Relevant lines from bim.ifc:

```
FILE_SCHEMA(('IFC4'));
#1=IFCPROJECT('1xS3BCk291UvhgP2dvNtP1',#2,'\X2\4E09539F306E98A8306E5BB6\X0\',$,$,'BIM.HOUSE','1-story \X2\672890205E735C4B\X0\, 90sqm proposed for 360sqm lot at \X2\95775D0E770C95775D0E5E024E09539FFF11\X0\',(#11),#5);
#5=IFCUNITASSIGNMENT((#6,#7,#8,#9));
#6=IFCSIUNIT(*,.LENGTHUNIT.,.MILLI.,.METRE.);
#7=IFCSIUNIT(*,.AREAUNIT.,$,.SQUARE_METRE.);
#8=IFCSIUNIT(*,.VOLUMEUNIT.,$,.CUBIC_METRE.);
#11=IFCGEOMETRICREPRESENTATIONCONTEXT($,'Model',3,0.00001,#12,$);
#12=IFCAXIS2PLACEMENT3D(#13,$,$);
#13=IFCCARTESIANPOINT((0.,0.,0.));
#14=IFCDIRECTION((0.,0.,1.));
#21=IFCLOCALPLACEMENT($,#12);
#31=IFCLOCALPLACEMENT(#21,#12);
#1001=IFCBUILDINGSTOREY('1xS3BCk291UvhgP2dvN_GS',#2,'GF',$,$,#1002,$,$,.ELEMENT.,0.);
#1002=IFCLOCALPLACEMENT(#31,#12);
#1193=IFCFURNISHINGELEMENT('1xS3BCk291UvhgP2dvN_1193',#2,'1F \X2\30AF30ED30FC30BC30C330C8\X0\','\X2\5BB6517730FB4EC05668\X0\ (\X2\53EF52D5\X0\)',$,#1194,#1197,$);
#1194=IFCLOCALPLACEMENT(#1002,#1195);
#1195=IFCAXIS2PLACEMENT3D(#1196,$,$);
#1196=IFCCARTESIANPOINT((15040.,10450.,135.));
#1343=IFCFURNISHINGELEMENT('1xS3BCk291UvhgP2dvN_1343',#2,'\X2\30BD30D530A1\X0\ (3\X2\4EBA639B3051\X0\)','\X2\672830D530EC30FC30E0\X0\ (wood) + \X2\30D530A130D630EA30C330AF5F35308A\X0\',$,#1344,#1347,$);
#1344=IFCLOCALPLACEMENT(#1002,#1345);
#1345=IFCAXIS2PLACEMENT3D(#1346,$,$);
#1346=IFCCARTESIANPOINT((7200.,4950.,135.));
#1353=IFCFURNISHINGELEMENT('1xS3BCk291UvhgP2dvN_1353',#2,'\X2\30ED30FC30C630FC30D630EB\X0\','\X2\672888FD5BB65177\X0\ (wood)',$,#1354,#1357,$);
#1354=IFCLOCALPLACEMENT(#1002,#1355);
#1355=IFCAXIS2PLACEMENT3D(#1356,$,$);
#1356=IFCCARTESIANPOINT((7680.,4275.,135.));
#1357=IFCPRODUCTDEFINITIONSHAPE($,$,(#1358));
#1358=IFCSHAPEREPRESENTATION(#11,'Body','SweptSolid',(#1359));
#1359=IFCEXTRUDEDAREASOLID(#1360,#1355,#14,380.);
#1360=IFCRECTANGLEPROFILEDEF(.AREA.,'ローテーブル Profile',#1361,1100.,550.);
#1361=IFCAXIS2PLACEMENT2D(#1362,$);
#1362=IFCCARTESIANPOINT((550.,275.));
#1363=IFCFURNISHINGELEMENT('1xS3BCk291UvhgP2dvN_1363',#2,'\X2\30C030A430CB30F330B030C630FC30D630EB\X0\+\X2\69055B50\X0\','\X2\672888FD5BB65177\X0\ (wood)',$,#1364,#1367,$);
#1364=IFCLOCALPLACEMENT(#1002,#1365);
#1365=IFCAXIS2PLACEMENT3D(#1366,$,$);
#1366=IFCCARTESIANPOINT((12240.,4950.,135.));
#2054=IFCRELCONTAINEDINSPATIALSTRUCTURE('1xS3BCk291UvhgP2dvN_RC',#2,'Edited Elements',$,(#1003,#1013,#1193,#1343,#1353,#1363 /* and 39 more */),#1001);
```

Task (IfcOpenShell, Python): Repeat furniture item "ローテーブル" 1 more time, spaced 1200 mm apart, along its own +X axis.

```python
import ifcopenshell
import ifcopenshell.api.geometry
import ifcopenshell.api.root
import ifcopenshell.util.element
import ifcopenshell.util.placement

model = ifcopenshell.open("bim.ifc")


def reuse_history(source, copy):
    """copy_class also copies each property set's owner history, people and application; keep the originals."""
    for rel in copy.IsDefinedBy:
        if rel.is_a("IfcRelDefinesByProperties") and (history := rel.RelatingPropertyDefinition.OwnerHistory):
            rel.RelatingPropertyDefinition.OwnerHistory = source.OwnerHistory
            ifcopenshell.util.element.remove_deep2(model, history)


source = model.by_id(1353)
base = ifcopenshell.util.placement.get_local_placement(source.ObjectPlacement)
step = base[:3, 0] * 1200.0

for i in range(1, 2):
    copy = ifcopenshell.api.root.copy_class(model, product=source)
    copy.Representation = ifcopenshell.util.element.copy_deep(
        model, source.Representation, exclude=["IfcGeometricRepresentationContext", "IfcRepresentationMap"]
    )
    reuse_history(source, copy)
    matrix = base.copy()
    matrix[:3, 3] += i * step
    print("added at", matrix[:3, 3].round(3) + 0.0)
    ifcopenshell.api.geometry.edit_object_placement(model, product=copy, matrix=matrix, is_si=False)

model.write("bim_rev.ifc")
```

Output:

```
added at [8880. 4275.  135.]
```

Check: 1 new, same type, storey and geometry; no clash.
